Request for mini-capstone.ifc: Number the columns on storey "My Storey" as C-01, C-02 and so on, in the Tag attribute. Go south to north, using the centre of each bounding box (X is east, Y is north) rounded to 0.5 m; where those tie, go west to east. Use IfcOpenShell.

First a look at what the model holds.

```python
import ifcopenshell
import ifcopenshell.util.element
import ifcopenshell.util.placement

model = ifcopenshell.open("mini-capstone.ifc")
print(model.schema)
storey = next(s for s in model.by_type("IfcBuildingStorey") if s.Name == "My Storey")
columns = [e for e in ifcopenshell.util.element.get_decomposition(storey) if e.is_a("IfcColumn")]
for e in sorted(columns, key=lambda e: e.id()):
    origin = ifcopenshell.util.placement.get_local_placement(e.ObjectPlacement)[:3, 3]
    print(e.id(), e.Tag, e.Name, origin.round(2) + 0.0, sep=" | ")
```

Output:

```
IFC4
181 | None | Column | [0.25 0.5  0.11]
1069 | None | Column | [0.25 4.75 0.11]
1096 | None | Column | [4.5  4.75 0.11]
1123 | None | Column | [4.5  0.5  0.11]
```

```python
import ifcopenshell
import ifcopenshell.geom
import ifcopenshell.util.element
import ifcopenshell.util.shape

model = ifcopenshell.open("mini-capstone.ifc")
settings = ifcopenshell.geom.settings()
settings.set("use-world-coords", True)


def centre(element):
    shape = ifcopenshell.geom.create_shape(settings, element)
    return ifcopenshell.util.shape.get_bbox_centroid(shape.geometry)


storey = next(s for s in model.by_type("IfcBuildingStorey") if s.Name == "My Storey")
columns = [e for e in ifcopenshell.util.element.get_decomposition(storey) if e.is_a("IfcColumn")]

# Insertion points can sit at a corner or the storey origin, so sort by the geometry (in metres).
centres = {e: centre(e) for e in columns}
columns.sort(key=lambda e: (round(centres[e][1] / 0.5), centres[e][0]))

for i, e in enumerate(columns, start=1):
    number = f"C-{i:02d}"
    e.Tag = number
    print(e.id(), number)

model.write("mini-capstone_updated.ifc")
```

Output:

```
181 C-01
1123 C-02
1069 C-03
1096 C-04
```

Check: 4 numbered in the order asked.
